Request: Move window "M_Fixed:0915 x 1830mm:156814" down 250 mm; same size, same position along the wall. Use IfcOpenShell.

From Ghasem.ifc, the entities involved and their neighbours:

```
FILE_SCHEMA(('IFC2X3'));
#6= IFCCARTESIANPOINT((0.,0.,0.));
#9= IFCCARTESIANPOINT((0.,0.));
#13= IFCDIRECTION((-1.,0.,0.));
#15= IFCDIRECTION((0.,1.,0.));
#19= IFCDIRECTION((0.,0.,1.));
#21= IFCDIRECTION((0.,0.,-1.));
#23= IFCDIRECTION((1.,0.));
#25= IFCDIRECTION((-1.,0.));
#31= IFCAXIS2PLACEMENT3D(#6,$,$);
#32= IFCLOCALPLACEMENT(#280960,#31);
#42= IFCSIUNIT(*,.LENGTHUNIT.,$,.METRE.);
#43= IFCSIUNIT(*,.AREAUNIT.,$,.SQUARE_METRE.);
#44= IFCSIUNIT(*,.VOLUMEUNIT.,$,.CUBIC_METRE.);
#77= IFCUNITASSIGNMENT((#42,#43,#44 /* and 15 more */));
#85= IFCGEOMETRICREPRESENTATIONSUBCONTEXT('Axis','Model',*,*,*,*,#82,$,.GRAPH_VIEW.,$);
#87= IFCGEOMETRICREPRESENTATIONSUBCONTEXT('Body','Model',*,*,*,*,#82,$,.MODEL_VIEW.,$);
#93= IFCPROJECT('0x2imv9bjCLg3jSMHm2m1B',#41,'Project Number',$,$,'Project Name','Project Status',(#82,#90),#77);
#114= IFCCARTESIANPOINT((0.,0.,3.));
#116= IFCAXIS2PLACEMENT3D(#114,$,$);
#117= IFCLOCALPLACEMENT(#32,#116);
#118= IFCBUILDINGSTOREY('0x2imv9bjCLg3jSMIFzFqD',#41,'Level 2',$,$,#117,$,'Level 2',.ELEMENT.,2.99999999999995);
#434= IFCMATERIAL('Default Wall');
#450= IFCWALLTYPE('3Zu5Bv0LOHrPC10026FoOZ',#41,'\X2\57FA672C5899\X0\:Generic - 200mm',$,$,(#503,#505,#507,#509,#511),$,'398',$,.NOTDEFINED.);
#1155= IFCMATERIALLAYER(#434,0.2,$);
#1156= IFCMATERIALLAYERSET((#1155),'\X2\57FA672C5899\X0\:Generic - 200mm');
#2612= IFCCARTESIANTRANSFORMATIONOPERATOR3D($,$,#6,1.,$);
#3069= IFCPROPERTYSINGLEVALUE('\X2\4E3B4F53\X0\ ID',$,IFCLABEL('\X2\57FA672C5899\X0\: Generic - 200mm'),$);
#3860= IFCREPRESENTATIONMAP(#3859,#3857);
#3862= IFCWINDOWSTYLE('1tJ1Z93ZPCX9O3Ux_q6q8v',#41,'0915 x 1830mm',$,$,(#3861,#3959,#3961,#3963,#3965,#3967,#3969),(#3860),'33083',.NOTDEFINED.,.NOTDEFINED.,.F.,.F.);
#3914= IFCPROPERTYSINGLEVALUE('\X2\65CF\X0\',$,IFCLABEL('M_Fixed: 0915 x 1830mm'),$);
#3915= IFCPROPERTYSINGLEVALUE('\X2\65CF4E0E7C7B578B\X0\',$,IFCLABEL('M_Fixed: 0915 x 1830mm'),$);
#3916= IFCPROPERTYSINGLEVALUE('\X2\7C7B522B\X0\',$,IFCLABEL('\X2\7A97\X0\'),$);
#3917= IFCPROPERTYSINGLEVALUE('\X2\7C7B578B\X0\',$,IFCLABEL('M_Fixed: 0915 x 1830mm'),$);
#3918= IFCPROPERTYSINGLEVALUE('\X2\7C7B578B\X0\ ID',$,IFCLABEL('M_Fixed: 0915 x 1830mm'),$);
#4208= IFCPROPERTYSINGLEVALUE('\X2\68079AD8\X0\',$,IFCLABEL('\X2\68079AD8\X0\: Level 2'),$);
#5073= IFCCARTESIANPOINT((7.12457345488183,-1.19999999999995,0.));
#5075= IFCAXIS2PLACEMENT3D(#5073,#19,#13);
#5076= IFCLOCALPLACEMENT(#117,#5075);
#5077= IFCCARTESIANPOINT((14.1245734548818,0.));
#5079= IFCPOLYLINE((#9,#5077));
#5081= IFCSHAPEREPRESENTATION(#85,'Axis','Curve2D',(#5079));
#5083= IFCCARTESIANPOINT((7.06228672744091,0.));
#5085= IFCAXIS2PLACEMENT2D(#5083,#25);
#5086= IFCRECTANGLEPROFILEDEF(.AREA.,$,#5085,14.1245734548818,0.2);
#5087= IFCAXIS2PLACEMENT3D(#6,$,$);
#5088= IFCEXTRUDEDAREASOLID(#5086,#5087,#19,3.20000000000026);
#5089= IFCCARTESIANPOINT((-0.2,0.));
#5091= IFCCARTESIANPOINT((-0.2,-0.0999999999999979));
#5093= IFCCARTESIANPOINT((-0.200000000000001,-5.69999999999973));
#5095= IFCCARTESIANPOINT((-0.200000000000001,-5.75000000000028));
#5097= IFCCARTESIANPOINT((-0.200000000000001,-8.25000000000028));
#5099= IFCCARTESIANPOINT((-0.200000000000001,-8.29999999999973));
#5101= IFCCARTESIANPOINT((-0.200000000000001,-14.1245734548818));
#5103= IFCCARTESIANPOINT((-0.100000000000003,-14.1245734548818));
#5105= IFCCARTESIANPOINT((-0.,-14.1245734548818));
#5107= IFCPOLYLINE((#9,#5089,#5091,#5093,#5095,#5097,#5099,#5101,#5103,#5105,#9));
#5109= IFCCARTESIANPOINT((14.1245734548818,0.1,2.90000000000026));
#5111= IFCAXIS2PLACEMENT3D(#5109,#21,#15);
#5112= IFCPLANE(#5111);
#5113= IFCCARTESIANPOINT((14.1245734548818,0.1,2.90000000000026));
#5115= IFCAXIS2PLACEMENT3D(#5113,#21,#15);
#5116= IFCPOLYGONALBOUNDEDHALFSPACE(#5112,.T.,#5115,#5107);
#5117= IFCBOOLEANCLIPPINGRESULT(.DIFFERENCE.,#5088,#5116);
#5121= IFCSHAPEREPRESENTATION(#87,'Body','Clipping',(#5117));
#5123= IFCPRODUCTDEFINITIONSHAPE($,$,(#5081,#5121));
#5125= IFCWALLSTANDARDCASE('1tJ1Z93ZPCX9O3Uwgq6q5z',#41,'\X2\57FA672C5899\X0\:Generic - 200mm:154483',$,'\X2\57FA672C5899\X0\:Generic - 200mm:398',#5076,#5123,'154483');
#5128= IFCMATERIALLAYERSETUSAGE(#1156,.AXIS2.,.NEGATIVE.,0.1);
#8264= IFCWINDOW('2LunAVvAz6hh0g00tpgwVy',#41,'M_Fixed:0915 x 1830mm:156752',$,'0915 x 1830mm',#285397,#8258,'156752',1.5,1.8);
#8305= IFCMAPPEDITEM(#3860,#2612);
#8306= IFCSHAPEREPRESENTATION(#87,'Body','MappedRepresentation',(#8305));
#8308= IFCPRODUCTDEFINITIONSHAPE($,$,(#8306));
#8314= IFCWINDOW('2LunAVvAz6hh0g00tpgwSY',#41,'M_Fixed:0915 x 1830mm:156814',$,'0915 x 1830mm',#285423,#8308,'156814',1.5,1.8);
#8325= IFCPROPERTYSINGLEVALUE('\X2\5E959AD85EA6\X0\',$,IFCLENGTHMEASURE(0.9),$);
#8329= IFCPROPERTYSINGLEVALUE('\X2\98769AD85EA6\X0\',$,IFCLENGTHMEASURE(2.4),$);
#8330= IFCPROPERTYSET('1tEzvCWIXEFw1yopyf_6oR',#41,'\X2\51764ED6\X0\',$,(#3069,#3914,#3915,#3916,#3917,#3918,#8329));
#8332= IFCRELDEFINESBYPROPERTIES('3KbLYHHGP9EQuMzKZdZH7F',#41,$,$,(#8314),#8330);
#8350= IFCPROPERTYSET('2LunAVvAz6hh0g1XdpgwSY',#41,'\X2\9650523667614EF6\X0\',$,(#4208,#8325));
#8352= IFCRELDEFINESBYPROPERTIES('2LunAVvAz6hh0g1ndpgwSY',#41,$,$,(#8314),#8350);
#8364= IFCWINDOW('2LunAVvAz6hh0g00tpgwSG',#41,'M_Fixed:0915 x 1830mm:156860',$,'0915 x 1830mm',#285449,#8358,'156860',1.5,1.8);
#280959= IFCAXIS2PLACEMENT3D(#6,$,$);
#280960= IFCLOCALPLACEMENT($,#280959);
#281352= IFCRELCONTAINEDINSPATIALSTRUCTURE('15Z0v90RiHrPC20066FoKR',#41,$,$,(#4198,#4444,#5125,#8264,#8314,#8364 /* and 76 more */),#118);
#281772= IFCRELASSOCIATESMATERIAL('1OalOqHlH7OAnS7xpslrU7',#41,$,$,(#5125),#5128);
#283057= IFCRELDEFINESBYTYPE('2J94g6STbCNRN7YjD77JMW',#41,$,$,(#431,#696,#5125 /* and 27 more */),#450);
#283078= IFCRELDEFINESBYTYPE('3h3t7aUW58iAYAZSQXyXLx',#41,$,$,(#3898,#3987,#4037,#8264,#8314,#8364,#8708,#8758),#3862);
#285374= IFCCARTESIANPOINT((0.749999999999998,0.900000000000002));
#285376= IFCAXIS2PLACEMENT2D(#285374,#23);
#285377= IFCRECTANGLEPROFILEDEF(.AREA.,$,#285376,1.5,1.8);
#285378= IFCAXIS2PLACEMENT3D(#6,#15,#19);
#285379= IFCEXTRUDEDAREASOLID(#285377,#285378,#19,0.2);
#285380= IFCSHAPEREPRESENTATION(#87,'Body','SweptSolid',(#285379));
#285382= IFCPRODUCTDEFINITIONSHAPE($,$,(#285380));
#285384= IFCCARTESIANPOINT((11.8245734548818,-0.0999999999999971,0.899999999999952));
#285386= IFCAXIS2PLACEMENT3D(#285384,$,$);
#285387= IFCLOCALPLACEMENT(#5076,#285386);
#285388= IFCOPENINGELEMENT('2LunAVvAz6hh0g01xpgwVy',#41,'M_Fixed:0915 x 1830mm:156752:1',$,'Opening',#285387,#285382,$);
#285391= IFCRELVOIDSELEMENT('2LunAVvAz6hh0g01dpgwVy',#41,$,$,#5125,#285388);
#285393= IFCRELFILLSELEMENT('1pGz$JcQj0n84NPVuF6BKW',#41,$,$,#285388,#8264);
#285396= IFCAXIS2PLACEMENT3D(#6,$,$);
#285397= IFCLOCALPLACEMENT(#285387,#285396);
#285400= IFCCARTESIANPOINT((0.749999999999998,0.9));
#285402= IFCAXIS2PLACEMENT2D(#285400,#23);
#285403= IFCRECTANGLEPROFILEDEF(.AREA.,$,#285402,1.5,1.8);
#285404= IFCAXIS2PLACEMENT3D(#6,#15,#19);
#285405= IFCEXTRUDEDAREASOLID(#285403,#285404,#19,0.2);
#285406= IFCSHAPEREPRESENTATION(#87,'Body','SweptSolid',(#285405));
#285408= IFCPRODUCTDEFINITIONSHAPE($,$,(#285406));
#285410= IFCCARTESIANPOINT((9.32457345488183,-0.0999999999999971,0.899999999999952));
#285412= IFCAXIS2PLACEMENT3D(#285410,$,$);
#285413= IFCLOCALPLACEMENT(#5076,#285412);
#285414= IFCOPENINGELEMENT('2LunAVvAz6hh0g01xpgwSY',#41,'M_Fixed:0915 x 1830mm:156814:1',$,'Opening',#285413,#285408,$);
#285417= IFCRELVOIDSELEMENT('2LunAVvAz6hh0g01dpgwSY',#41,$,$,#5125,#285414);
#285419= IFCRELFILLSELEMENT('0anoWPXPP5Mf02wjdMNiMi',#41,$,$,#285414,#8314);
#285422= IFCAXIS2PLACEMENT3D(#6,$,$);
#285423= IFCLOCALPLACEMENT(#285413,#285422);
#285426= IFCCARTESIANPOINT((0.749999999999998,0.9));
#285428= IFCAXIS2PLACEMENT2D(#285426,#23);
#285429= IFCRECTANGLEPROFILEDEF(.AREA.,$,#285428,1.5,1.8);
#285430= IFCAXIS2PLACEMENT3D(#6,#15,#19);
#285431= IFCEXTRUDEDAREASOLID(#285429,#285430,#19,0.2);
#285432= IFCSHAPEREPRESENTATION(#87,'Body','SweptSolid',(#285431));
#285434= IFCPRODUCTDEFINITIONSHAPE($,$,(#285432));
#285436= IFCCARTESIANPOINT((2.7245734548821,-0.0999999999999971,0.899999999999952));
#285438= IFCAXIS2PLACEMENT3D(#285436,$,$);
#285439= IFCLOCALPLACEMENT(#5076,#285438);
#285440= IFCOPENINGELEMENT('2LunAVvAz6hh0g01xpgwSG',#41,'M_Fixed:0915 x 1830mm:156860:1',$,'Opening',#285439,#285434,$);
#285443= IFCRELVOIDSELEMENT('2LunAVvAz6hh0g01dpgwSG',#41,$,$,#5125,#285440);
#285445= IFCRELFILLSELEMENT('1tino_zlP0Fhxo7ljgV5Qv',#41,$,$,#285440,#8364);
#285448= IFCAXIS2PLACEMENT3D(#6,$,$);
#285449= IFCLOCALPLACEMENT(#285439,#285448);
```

```python
import numpy as np
import ifcopenshell
import ifcopenshell.api.geometry
import ifcopenshell.api.pset
import ifcopenshell.util.element
import ifcopenshell.util.placement
import ifcopenshell.util.unit

model = ifcopenshell.open("Ghasem.ifc")
unit_scale = ifcopenshell.util.unit.calculate_unit_scale(model)

window = model.by_guid("2LunAVvAz6hh0g00tpgwSY")
opening = window.FillsVoids[0].RelatingOpeningElement
dz = -0.25 / unit_scale

shift = np.array([0.0, 0.0, dz])
# The window is placed relative to its opening, so it follows when the opening moves.
matrix = ifcopenshell.util.placement.get_local_placement(opening.ObjectPlacement)
matrix[:3, 3] += shift
ifcopenshell.api.geometry.edit_object_placement(
    model, product=opening, matrix=matrix, is_si=False, should_transform_children=True
)

# Keep the stored heights in step.
pset = model.by_id(ifcopenshell.util.element.get_pset(window, "其他", should_inherit=False)["id"])
ifcopenshell.api.pset.edit_pset(model, pset=pset, properties={
    "顶高度": model.create_entity("IfcLengthMeasure", ifcopenshell.util.element.get_pset(window, "其他", "顶高度") + dz),
})
pset = model.by_id(ifcopenshell.util.element.get_pset(window, "限制条件", should_inherit=False)["id"])
ifcopenshell.api.pset.edit_pset(model, pset=pset, properties={
    "底高度": model.create_entity("IfcLengthMeasure", ifcopenshell.util.element.get_pset(window, "限制条件", "底高度") + dz),
})

print(f"moved by {dz * unit_scale:+.3f} m")

model.write("Ghasem-out.ifc")
```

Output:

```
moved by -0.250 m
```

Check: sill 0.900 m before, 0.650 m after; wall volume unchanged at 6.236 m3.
